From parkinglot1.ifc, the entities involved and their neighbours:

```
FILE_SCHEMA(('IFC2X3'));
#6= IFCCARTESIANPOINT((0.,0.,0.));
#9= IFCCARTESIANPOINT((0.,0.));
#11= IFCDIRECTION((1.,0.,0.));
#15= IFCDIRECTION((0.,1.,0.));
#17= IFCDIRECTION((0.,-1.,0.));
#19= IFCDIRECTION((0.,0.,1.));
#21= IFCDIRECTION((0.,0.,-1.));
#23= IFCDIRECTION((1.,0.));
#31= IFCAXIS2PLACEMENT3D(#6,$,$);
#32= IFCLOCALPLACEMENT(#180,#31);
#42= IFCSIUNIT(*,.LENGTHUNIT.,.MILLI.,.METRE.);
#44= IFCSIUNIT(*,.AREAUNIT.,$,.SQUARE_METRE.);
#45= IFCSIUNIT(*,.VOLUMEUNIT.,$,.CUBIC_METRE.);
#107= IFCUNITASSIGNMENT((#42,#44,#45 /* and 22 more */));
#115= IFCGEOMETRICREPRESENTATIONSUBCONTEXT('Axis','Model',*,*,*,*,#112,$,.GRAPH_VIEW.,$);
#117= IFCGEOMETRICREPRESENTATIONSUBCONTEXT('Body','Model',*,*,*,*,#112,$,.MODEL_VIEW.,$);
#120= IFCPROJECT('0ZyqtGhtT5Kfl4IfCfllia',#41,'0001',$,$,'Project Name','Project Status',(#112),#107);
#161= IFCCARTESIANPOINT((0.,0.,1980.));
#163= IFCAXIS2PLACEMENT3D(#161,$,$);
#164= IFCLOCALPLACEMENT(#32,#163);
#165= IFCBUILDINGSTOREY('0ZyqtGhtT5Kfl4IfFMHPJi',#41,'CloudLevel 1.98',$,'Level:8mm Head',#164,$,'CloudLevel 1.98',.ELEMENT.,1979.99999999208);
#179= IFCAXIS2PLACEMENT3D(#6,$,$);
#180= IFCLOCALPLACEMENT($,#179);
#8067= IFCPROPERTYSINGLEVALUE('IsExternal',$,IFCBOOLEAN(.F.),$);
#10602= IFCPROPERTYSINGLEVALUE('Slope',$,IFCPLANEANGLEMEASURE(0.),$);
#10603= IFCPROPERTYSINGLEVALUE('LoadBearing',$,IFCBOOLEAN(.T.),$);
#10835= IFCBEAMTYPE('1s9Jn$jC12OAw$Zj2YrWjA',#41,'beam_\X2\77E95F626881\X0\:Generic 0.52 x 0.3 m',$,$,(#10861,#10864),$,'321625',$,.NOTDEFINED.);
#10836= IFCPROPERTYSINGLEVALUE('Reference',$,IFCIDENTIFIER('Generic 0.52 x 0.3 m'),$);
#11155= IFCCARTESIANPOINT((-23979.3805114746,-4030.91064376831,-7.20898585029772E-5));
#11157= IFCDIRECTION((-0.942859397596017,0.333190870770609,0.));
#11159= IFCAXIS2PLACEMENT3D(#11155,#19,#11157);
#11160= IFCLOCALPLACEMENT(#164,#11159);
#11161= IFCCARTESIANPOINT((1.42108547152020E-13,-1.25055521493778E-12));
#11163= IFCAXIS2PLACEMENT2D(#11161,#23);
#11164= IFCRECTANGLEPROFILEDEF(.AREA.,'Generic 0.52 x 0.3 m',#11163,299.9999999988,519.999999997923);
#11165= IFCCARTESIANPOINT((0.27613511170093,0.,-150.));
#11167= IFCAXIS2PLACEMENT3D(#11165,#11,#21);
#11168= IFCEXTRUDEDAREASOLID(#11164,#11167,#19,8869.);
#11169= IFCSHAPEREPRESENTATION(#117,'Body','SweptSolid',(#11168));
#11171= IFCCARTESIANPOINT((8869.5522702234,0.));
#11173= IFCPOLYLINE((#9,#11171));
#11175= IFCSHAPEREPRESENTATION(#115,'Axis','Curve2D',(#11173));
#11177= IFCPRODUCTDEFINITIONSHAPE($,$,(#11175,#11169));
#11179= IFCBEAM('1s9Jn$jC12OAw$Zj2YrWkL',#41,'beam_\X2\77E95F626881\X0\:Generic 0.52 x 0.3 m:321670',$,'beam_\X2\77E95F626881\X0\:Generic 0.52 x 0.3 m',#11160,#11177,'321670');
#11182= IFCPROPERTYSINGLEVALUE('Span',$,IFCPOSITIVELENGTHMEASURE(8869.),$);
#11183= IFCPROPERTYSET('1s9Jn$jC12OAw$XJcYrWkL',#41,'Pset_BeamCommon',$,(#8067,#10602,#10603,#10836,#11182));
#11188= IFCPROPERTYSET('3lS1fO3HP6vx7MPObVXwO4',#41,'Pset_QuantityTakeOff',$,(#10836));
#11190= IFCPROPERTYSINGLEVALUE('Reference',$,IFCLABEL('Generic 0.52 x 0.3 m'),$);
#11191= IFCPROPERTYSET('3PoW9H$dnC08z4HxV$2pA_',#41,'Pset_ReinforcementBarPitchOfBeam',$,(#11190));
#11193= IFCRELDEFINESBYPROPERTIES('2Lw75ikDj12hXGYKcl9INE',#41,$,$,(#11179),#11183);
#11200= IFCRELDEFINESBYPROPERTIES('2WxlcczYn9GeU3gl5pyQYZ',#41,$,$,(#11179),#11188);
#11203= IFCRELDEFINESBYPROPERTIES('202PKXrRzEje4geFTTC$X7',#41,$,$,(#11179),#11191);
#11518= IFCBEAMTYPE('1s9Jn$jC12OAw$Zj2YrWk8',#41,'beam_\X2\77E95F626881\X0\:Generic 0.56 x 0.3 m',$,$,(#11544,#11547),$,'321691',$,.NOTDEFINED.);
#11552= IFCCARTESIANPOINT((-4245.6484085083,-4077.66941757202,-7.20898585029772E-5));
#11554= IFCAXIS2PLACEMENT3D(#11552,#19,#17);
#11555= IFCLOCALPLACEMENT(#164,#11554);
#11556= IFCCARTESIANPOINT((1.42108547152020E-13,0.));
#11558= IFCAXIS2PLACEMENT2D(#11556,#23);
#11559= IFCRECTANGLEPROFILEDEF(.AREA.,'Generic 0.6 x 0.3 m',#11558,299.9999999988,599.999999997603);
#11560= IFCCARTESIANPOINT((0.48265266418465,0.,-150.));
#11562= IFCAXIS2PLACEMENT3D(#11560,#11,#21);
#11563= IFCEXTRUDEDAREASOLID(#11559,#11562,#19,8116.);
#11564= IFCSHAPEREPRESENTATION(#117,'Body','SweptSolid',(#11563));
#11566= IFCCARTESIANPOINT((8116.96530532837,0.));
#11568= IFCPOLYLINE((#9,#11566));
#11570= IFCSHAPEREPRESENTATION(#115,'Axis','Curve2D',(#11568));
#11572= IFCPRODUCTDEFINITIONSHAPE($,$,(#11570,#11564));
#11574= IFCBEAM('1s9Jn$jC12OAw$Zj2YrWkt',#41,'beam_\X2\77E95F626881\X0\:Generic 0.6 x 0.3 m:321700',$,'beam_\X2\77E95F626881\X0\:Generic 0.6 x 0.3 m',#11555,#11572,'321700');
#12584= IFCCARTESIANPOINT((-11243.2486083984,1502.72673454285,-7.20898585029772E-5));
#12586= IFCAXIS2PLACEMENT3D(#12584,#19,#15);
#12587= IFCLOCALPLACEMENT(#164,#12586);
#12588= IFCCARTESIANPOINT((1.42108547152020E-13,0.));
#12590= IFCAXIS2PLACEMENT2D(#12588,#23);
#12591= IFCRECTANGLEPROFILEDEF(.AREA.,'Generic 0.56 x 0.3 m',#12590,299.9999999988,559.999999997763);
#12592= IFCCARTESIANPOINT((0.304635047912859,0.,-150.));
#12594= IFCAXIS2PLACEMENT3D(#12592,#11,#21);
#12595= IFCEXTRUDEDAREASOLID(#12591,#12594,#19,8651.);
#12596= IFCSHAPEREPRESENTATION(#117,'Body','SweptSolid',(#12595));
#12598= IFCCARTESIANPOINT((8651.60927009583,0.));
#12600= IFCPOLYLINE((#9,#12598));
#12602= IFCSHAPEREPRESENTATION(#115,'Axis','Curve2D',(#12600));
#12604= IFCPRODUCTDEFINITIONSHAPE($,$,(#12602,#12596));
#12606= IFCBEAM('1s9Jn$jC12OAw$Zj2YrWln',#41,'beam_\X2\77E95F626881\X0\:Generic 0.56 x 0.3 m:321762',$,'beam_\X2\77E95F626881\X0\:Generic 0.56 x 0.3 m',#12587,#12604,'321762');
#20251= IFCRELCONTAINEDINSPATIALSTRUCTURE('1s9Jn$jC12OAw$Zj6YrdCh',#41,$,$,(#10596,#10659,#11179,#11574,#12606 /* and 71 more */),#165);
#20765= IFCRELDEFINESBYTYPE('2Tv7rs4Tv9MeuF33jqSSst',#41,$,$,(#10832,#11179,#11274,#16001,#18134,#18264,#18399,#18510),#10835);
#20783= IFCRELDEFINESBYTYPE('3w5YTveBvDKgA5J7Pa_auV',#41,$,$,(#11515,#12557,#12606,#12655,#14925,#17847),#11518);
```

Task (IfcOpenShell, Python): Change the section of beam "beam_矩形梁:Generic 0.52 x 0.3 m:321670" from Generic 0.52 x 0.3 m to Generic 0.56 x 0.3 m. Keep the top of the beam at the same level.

```python
import ifcopenshell
import ifcopenshell.api.pset
import ifcopenshell.api.type
import ifcopenshell.util.element
import ifcopenshell.util.representation

model = ifcopenshell.open("parkinglot1.ifc")

member = model.by_id(11179)
source = next(p for p in model.by_type("IfcRectangleProfileDef") if p.ProfileName == "Generic 0.56 x 0.3 m")

body = ifcopenshell.util.representation.get_representation(member, "Model", "Body")
solid = body.Items[0]
old_profile = solid.SweptArea

# Copy the section's sizes but keep this member's own profile position.
profile = ifcopenshell.util.element.copy(model, source)
# Profiles are centred, so shift by half the change in depth to hold the top.
shift = (old_profile.XDim - profile.XDim) / 2
x, y = old_profile.Position.Location.Coordinates
up = (-1.0, 0.0)  # upwards, in the solid's own plane
location = model.createIfcCartesianPoint((x + up[0] * shift, y + up[1] * shift))
profile.Position = model.createIfcAxis2Placement2D(location, old_profile.Position.RefDirection)
solid.SweptArea = profile
if not model.get_total_inverses(old_profile):
    ifcopenshell.util.element.remove_deep2(model, old_profile)

new_type = model.by_id(11518)
ifcopenshell.api.type.assign_type(
    model, related_objects=[member], relating_type=new_type, should_map_representations=False
)
member.Name = member.Name.replace("Generic 0.52 x 0.3 m", "Generic 0.56 x 0.3 m")
member.ObjectType = "beam_矩形梁:Generic 0.56 x 0.3 m"
pset = model.by_id(ifcopenshell.util.element.get_pset(member, "Pset_BeamCommon", should_inherit=False)["id"])
ifcopenshell.api.pset.edit_pset(model, pset=pset, properties={"Reference": "Generic 0.56 x 0.3 m"})
pset = model.by_id(ifcopenshell.util.element.get_pset(member, "Pset_QuantityTakeOff", should_inherit=False)["id"])
ifcopenshell.api.pset.edit_pset(model, pset=pset, properties={"Reference": "Generic 0.56 x 0.3 m"})
pset = model.by_id(ifcopenshell.util.element.get_pset(member, "Pset_ReinforcementBarPitchOfBeam", should_inherit=False)["id"])
ifcopenshell.api.pset.edit_pset(model, pset=pset, properties={"Reference": "Generic 0.56 x 0.3 m"})

print(solid.SweptArea)

model.write("parkinglot1_updated.ifc")
```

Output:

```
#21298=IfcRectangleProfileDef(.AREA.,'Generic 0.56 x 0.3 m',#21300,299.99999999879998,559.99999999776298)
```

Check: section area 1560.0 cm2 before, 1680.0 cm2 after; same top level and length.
